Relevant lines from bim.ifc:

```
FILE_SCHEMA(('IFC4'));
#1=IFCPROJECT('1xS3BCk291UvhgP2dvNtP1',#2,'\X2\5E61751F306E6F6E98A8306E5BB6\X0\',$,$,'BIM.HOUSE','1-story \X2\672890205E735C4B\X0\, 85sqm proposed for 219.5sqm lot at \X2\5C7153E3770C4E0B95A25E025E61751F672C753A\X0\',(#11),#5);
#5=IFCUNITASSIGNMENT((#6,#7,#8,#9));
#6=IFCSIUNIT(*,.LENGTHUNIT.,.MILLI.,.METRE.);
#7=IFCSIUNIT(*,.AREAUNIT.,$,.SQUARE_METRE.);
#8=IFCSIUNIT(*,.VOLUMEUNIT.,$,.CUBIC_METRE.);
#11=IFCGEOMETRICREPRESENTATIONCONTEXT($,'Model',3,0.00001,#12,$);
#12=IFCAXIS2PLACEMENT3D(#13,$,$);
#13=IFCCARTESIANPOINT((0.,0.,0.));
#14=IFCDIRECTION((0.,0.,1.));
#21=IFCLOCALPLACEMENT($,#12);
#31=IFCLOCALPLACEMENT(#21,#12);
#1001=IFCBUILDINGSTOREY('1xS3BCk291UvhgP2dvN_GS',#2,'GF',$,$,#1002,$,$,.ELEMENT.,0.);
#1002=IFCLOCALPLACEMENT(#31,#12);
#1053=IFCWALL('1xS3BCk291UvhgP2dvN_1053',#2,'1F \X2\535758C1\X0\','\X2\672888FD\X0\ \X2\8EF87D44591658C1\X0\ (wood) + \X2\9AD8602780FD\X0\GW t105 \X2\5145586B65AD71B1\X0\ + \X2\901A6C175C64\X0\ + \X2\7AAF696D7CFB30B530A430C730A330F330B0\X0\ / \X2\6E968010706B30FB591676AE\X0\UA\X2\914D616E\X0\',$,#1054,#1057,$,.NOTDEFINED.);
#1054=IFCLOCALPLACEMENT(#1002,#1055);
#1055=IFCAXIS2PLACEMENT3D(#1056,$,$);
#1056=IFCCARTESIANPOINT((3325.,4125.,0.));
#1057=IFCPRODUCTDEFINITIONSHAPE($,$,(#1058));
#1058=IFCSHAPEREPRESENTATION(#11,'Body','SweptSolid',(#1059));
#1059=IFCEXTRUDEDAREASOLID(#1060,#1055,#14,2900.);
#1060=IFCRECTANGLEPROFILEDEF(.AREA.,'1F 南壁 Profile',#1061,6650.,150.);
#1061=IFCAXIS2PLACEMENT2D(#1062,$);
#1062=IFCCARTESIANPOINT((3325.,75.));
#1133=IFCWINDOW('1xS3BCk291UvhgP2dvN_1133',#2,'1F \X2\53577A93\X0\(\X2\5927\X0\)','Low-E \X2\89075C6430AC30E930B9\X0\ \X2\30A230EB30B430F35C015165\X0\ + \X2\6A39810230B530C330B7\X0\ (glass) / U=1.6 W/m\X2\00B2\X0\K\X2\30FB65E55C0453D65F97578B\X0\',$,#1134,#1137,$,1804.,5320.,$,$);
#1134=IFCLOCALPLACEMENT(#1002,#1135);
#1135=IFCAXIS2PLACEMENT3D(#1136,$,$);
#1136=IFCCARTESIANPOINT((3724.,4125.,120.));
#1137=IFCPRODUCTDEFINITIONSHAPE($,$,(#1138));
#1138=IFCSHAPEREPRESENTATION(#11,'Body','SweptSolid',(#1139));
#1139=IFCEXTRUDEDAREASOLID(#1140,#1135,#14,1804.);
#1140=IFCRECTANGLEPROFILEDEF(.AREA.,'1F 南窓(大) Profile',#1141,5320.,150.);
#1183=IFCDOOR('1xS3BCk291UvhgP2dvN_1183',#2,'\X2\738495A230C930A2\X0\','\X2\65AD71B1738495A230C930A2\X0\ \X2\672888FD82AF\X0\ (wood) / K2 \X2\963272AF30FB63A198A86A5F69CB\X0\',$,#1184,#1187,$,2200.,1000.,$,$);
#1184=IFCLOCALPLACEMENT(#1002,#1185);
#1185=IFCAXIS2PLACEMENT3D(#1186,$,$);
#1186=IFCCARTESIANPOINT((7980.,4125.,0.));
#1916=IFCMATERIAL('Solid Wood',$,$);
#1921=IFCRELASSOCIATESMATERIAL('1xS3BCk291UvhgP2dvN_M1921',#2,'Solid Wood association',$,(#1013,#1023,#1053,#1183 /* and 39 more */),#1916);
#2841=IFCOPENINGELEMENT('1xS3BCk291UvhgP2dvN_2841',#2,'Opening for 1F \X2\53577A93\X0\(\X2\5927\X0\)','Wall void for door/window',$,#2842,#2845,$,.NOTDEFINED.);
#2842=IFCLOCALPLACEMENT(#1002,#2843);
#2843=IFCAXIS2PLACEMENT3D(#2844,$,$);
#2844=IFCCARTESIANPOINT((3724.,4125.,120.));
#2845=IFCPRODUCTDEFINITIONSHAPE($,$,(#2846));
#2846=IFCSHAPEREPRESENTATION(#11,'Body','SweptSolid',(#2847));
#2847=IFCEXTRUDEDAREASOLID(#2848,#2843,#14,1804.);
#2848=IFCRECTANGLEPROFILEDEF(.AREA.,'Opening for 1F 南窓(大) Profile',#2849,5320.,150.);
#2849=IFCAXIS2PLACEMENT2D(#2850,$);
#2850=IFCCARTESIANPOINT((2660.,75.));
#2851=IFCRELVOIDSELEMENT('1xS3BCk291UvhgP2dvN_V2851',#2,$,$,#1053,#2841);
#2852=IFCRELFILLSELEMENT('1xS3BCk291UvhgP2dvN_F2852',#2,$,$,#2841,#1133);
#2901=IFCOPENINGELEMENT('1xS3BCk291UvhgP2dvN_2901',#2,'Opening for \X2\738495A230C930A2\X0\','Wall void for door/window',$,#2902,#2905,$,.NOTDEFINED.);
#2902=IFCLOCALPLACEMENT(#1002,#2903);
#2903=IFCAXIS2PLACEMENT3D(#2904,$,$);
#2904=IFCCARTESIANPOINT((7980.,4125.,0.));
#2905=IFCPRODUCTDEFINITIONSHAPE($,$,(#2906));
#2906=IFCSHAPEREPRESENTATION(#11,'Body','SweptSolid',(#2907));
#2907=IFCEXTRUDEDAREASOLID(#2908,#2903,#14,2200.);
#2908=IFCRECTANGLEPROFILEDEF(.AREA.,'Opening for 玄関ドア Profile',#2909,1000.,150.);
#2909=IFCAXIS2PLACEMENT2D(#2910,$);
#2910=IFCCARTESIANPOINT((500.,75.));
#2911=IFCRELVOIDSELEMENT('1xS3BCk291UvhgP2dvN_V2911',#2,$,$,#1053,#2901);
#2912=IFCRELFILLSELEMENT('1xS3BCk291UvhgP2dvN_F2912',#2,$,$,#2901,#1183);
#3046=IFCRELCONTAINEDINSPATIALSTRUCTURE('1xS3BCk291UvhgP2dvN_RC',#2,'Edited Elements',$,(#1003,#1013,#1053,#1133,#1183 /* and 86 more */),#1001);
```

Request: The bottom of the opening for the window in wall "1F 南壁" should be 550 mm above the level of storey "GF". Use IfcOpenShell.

```python
import numpy as np
import ifcopenshell
import ifcopenshell.api.geometry
import ifcopenshell.geom
import ifcopenshell.util.element
import ifcopenshell.util.placement
import ifcopenshell.util.shape
import ifcopenshell.util.unit

model = ifcopenshell.open("bim.ifc")
unit_scale = ifcopenshell.util.unit.calculate_unit_scale(model)

window = model.by_id(1133)
opening = window.FillsVoids[0].RelatingOpeningElement
storey = ifcopenshell.util.element.get_container(window, ifc_class="IfcBuildingStorey")
level = ifcopenshell.util.placement.get_local_placement(storey.ObjectPlacement)[2, 3]

# The opening's origin need not be at the sill, so measure its lowest point.
shape = ifcopenshell.geom.create_shape(ifcopenshell.geom.settings(), opening)
bottom = ifcopenshell.util.shape.get_shape_bottom_elevation(shape, shape.geometry) / unit_scale
dz = level + 550.0 - bottom

shift = np.array([0.0, 0.0, dz])
# The window is not placed relative to its opening, so move both.
for product in (opening, window):
    matrix = ifcopenshell.util.placement.get_local_placement(product.ObjectPlacement)
    matrix[:3, 3] += shift
    ifcopenshell.api.geometry.edit_object_placement(model, product=product, matrix=matrix, is_si=False)

print(f"moved by {dz * unit_scale:+.3f} m")

model.write("bim-out.ifc")
```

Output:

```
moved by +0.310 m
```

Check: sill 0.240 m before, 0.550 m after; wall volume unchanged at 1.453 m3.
